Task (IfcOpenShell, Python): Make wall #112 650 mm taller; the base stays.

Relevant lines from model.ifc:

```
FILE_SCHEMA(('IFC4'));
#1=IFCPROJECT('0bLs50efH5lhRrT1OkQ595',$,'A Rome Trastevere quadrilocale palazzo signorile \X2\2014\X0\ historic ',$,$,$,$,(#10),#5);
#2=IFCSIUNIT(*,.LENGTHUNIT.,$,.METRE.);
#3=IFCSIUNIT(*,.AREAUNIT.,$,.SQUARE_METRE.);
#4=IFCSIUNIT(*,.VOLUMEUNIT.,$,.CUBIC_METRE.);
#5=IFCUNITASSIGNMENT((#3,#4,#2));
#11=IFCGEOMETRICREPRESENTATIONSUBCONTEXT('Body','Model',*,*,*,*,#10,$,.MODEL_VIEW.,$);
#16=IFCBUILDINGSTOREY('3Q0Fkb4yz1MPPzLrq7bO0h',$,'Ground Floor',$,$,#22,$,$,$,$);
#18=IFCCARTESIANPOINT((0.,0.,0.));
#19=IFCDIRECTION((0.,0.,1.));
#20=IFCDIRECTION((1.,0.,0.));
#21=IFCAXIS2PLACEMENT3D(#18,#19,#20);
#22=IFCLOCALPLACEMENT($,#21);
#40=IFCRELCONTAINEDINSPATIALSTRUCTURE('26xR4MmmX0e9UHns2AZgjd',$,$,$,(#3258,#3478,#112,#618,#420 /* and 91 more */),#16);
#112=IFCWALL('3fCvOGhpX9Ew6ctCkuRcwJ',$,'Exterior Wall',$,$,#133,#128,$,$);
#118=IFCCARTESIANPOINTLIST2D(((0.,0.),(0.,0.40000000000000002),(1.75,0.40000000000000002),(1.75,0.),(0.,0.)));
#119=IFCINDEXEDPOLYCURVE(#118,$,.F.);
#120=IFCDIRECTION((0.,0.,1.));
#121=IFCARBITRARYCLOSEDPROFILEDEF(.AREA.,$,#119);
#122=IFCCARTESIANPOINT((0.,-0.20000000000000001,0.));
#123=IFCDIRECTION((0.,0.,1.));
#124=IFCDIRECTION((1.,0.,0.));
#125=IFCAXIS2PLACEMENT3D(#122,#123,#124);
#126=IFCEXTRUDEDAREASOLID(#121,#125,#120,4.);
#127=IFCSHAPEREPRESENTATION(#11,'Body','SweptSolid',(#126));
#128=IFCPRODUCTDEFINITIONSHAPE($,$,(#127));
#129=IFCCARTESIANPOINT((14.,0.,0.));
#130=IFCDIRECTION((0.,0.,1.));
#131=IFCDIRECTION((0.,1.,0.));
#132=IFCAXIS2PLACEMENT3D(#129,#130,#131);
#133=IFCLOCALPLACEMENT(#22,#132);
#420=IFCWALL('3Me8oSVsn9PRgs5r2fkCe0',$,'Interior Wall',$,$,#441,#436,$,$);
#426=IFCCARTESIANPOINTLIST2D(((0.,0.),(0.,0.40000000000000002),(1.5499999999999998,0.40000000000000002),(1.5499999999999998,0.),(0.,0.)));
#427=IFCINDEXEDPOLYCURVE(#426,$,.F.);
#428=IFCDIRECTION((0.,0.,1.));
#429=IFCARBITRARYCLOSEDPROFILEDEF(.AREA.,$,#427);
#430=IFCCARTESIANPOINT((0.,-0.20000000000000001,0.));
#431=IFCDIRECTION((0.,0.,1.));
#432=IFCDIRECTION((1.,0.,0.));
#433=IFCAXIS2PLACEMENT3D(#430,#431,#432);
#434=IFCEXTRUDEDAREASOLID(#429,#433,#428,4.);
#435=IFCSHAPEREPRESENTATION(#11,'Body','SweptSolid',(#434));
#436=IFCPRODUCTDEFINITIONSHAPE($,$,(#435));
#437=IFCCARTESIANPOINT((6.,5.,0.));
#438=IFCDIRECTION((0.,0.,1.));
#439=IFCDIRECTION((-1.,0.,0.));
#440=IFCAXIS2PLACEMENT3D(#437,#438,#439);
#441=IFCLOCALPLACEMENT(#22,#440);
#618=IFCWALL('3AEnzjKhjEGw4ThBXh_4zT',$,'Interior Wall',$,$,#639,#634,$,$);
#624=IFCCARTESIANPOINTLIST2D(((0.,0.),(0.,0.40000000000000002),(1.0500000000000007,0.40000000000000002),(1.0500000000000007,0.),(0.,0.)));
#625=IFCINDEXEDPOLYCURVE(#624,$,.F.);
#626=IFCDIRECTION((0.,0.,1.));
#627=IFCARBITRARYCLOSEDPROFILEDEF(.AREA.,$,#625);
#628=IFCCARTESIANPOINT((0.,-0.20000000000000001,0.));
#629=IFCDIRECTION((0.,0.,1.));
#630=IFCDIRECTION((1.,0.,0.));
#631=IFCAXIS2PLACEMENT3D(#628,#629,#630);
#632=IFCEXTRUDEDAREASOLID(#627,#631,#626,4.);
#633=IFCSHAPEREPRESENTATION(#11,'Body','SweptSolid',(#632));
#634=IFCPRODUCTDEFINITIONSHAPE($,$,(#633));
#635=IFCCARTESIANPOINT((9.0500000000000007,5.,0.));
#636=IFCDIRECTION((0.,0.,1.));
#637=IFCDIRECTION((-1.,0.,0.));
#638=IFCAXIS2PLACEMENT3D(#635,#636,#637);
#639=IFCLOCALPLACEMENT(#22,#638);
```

```python
import ifcopenshell
import ifcopenshell.geom
import ifcopenshell.util.representation
import ifcopenshell.util.shape
import ifcopenshell.util.unit

model = ifcopenshell.open("model.ifc")
unit_scale = ifcopenshell.util.unit.calculate_unit_scale(model)
settings = ifcopenshell.geom.settings()


def volume(element):
    """Net volume in cubic metres, openings subtracted."""
    shape = ifcopenshell.geom.create_shape(settings, element)
    return ifcopenshell.util.shape.get_volume(shape.geometry)


wall = model.by_id(112)
before = volume(wall)

body = ifcopenshell.util.representation.get_representation(wall, "Model", "Body")
solid = body.Items[0]
old_height = solid.Depth
solid.Depth += 0.65 / unit_scale
after = volume(wall)

print(f"height {old_height:g} -> {solid.Depth:g}, volume {before:.3f} -> {after:.3f} m3")

model.write("model_rev.ifc")
```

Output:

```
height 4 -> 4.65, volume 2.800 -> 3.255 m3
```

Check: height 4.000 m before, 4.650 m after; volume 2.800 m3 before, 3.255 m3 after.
